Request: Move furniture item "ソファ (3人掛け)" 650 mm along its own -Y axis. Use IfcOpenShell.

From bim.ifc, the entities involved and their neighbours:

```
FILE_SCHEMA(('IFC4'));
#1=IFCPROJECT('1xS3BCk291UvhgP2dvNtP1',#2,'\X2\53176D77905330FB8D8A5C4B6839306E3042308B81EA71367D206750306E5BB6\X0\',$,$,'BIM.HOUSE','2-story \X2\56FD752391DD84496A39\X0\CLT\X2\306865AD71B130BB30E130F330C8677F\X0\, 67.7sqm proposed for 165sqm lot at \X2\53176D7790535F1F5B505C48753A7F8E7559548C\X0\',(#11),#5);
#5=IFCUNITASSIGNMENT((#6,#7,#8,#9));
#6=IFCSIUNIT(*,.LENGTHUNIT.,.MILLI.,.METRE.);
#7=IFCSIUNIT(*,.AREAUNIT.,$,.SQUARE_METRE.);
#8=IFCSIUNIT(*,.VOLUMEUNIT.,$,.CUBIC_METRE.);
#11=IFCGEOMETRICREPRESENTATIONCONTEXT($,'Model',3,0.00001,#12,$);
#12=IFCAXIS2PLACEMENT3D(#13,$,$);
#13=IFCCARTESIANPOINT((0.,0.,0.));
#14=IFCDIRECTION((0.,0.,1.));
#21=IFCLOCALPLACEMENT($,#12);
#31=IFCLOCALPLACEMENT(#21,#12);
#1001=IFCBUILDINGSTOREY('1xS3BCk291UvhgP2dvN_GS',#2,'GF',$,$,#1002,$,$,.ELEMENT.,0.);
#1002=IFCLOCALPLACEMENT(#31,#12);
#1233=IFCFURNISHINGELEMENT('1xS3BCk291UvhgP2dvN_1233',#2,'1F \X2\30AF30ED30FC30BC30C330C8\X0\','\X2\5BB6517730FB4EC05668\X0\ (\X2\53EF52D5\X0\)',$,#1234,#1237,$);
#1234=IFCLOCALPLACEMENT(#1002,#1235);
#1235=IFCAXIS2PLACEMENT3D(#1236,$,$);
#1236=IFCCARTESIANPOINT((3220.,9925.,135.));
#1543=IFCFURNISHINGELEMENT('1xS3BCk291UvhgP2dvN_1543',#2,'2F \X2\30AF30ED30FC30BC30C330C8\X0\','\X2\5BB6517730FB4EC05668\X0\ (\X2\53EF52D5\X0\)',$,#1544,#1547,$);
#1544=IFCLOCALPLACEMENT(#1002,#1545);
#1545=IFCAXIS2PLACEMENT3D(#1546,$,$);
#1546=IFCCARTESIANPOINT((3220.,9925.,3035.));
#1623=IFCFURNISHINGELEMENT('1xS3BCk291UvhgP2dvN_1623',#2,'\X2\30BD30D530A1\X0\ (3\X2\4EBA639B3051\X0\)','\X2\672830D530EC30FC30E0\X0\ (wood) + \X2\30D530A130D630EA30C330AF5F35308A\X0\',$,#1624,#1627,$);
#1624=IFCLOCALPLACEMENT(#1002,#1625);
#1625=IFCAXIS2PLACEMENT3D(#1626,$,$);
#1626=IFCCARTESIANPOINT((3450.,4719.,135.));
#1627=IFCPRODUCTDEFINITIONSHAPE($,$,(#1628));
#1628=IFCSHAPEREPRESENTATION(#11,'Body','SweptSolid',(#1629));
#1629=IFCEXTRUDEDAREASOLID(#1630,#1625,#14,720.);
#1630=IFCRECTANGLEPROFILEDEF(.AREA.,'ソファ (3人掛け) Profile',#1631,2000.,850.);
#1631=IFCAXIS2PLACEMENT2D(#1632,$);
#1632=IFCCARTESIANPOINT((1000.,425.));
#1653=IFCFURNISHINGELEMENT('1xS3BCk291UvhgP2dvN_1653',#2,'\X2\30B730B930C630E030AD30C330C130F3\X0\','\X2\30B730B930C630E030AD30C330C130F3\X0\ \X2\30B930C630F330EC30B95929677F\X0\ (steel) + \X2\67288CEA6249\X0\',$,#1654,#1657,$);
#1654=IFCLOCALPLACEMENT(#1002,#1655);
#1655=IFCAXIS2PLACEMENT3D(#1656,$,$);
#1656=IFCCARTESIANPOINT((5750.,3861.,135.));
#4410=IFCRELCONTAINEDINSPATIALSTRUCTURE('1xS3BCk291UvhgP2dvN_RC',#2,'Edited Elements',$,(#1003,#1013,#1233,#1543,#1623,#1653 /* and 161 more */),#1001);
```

```python
import ifcopenshell
import ifcopenshell.api.geometry
import ifcopenshell.util.placement
import ifcopenshell.util.unit

model = ifcopenshell.open("bim.ifc")
unit_scale = ifcopenshell.util.unit.calculate_unit_scale(model)

item = model.by_guid("1xS3BCk291UvhgP2dvN_1623")
matrix = ifcopenshell.util.placement.get_local_placement(item.ObjectPlacement)
matrix[:3, 3] -= matrix[:3, 1] * 0.65 / unit_scale
ifcopenshell.api.geometry.edit_object_placement(model, product=item, matrix=matrix, is_si=False)

print(ifcopenshell.util.placement.get_local_placement(item.ObjectPlacement).round(3) + 0.0)

model.write("bim_v2.ifc")
```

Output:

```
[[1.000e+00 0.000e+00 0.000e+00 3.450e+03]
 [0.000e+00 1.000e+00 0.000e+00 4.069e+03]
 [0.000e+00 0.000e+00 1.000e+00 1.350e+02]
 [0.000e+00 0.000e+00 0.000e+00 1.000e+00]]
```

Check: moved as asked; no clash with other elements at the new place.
